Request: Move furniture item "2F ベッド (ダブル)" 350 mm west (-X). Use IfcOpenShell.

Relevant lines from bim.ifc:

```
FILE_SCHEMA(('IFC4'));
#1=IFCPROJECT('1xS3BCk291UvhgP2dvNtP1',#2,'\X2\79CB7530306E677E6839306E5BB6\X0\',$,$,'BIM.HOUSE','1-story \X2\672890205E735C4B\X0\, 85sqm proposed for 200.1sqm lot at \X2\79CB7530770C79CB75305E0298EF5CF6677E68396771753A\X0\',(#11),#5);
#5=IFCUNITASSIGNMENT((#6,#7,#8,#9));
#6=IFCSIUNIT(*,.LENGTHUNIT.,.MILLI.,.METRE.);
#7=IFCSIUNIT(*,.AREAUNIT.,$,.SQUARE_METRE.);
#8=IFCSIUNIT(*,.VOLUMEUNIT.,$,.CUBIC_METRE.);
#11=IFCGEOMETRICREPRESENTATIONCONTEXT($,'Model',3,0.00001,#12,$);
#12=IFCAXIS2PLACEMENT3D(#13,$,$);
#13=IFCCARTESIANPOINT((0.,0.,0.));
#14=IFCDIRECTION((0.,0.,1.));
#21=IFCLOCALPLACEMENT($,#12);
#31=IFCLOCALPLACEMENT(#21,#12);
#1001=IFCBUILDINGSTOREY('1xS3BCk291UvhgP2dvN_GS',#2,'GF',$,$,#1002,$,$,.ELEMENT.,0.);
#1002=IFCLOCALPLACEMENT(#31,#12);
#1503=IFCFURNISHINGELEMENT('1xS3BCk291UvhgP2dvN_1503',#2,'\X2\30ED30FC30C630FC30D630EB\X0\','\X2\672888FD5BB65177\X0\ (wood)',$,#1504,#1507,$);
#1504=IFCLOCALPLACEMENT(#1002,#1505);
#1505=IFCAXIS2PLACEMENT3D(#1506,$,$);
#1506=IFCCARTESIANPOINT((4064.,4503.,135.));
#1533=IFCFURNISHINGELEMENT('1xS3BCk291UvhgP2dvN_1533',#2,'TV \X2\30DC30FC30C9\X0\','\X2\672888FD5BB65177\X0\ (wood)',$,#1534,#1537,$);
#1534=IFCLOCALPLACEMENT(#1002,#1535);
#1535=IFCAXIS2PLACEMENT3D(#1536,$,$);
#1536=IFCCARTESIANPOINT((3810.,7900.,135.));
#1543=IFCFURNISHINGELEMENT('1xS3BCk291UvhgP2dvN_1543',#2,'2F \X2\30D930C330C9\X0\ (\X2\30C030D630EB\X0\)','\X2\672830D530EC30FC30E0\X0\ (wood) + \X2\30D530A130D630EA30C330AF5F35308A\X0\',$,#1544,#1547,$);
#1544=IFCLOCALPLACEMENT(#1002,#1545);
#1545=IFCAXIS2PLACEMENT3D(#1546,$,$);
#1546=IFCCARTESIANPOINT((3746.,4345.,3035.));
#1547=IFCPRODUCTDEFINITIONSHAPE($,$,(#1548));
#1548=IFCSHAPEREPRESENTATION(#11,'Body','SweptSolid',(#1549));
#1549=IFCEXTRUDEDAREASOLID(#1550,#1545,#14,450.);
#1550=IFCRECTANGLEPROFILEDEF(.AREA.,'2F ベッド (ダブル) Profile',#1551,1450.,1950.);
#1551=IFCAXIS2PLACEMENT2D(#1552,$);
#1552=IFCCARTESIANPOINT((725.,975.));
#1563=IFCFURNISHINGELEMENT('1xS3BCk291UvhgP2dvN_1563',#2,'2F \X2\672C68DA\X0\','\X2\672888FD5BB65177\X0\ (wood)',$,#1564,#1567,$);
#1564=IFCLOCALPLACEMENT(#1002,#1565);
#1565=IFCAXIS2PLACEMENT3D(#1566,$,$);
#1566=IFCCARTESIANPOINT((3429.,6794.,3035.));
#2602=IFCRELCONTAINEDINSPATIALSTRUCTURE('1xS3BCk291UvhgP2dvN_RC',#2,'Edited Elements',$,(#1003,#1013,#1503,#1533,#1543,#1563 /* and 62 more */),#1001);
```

```python
import ifcopenshell
import ifcopenshell.api.geometry
import ifcopenshell.util.placement
import ifcopenshell.util.unit

model = ifcopenshell.open("bim.ifc")
unit_scale = ifcopenshell.util.unit.calculate_unit_scale(model)

item = model.by_id(1543)
matrix = ifcopenshell.util.placement.get_local_placement(item.ObjectPlacement)
matrix[0, 3] -= 0.35 / unit_scale
ifcopenshell.api.geometry.edit_object_placement(model, product=item, matrix=matrix, is_si=False)

print(ifcopenshell.util.placement.get_local_placement(item.ObjectPlacement).round(3) + 0.0)

model.write("bim-out.ifc")
```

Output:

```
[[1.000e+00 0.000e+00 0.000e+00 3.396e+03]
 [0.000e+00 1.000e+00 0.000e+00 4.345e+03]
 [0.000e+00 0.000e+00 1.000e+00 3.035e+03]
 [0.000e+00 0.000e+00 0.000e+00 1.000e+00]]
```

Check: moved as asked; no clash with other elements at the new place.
